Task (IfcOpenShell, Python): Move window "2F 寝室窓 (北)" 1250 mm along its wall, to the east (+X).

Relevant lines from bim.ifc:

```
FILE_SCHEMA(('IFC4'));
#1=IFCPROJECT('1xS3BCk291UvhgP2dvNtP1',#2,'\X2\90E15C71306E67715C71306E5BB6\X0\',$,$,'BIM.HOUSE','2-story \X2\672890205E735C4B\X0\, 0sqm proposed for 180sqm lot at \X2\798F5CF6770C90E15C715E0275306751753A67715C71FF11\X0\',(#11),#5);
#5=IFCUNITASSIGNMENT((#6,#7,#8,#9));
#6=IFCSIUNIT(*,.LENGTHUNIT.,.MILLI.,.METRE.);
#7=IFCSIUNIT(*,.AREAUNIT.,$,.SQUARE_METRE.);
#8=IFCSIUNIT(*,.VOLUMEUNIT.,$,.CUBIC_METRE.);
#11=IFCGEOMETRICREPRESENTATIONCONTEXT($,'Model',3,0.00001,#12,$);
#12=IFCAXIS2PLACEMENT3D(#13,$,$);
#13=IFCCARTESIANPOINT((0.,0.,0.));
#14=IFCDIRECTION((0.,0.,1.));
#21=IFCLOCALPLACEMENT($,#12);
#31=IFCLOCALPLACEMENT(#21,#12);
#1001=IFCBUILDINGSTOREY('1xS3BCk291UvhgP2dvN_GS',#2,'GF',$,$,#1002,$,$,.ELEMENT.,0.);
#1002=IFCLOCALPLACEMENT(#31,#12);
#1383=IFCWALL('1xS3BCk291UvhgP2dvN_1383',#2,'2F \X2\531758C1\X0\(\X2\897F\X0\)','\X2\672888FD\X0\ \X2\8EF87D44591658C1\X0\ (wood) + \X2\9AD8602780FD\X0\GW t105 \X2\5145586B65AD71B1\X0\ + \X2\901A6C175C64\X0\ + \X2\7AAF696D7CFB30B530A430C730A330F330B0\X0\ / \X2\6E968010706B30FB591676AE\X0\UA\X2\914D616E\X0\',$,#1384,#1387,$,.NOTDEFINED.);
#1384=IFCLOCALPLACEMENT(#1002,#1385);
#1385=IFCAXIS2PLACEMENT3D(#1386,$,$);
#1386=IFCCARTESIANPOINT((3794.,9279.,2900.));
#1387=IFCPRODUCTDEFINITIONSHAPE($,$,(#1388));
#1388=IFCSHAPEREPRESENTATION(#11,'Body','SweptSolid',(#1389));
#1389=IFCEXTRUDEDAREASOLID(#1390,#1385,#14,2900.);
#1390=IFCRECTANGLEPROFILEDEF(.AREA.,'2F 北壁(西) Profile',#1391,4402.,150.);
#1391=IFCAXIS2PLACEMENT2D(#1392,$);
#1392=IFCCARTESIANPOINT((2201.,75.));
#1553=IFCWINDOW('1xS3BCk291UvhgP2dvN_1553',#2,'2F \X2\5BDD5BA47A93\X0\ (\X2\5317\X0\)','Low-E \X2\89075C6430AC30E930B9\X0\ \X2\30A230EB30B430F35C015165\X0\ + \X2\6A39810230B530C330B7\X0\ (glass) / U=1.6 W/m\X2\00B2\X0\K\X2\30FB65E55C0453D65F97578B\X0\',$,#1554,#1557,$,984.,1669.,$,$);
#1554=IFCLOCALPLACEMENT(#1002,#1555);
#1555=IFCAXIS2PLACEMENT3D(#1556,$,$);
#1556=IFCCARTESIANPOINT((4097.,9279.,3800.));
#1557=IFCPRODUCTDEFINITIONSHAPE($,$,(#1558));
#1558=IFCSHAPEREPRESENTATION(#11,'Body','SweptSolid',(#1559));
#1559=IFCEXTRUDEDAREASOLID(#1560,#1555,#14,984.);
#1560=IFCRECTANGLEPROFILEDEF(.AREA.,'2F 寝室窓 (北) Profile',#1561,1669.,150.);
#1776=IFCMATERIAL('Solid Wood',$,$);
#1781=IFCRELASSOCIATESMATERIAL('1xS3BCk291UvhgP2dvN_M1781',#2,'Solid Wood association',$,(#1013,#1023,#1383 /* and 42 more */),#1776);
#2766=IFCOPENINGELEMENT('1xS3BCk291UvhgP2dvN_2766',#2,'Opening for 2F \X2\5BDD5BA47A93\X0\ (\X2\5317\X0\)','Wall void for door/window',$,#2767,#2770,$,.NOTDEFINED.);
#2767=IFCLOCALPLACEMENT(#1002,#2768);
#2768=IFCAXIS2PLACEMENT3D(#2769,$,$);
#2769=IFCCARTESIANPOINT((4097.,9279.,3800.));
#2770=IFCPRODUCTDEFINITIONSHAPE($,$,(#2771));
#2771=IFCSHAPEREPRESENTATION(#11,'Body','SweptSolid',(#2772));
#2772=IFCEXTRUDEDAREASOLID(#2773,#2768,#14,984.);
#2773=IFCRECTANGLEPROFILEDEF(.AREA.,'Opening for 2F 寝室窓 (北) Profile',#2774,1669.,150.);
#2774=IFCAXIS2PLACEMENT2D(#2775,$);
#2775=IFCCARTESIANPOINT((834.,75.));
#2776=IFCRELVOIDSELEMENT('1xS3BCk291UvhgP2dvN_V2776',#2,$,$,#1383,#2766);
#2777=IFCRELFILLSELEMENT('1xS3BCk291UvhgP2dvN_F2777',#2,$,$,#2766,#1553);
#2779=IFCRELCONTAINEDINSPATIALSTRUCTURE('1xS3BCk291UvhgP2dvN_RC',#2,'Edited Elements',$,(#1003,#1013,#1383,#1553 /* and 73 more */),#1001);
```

```python
import ifcopenshell
import ifcopenshell.api.geometry
import ifcopenshell.util.placement

model = ifcopenshell.open("bim.ifc")

window = model.by_id(1553)
opening = window.FillsVoids[0].RelatingOpeningElement
wall = opening.VoidsElements[0].RelatingBuildingElement

wall_matrix = ifcopenshell.util.placement.get_local_placement(wall.ObjectPlacement)
shift = wall_matrix[:3, 0] * 1250.0
before = ifcopenshell.util.placement.get_local_placement(window.ObjectPlacement)[:3, 3].copy()

# The window is not placed relative to its opening, so move both.
for product in (opening, window):
    matrix = ifcopenshell.util.placement.get_local_placement(product.ObjectPlacement)
    matrix[:3, 3] += shift
    ifcopenshell.api.geometry.edit_object_placement(model, product=product, matrix=matrix, is_si=False)

after = ifcopenshell.util.placement.get_local_placement(window.ObjectPlacement)[:3, 3]
print("window moved by", (after - before).round(3) + 0.0)

model.write("bim_v2.ifc")
```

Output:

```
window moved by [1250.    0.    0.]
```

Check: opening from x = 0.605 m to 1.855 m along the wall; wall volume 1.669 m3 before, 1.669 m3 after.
